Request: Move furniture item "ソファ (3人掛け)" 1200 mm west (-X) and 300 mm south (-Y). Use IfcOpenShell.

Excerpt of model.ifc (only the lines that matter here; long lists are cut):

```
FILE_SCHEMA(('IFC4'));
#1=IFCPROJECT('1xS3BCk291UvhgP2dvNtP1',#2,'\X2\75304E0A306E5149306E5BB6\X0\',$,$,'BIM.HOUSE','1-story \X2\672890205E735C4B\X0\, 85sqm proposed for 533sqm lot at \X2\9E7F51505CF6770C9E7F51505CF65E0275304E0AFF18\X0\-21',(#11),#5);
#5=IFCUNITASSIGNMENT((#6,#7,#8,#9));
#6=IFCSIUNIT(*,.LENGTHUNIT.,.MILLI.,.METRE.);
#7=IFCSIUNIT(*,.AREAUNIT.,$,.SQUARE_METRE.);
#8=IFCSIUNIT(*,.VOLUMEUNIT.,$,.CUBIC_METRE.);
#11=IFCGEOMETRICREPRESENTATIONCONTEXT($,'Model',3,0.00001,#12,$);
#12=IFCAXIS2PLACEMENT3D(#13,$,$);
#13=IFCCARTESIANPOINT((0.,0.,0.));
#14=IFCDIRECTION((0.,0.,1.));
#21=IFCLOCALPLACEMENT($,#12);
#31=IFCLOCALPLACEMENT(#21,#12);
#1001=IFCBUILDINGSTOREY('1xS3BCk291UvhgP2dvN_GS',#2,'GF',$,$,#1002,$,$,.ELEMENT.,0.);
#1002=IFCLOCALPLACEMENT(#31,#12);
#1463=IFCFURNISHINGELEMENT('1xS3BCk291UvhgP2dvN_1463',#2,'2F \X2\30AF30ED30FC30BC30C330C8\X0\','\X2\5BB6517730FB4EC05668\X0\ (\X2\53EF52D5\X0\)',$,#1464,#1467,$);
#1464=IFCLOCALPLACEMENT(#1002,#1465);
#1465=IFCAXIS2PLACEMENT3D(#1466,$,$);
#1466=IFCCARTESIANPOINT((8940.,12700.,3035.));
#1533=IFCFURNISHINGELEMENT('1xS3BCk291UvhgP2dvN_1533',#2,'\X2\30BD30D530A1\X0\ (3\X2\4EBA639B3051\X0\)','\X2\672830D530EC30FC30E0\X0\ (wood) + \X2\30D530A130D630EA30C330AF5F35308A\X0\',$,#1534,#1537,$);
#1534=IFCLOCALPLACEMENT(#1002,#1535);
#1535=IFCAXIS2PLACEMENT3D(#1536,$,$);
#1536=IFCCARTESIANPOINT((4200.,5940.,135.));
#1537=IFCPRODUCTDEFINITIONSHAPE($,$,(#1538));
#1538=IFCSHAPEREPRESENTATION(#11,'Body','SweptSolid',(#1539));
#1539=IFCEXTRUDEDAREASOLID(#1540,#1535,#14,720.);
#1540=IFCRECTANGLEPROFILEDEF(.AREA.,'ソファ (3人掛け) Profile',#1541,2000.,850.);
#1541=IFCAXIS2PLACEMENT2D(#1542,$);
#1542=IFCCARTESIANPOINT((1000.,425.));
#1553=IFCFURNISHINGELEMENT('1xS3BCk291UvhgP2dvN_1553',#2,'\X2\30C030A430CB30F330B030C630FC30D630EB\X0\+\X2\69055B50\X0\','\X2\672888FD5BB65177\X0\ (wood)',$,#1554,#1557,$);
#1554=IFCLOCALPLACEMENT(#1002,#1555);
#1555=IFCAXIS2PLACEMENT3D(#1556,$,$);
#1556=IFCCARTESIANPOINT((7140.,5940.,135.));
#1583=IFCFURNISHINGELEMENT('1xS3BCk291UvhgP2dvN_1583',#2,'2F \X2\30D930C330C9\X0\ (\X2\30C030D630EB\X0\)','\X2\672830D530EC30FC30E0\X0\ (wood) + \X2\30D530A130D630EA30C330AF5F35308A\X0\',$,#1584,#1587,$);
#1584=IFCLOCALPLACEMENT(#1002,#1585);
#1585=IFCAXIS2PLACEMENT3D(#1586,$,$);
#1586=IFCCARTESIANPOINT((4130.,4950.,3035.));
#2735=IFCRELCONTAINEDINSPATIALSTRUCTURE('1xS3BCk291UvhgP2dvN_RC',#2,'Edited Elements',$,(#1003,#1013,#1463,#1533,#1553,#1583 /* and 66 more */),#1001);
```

```python
import ifcopenshell
import ifcopenshell.api.geometry
import ifcopenshell.util.placement
import ifcopenshell.util.unit

model = ifcopenshell.open("model.ifc")
unit_scale = ifcopenshell.util.unit.calculate_unit_scale(model)

item = model.by_guid("1xS3BCk291UvhgP2dvN_1533")
matrix = ifcopenshell.util.placement.get_local_placement(item.ObjectPlacement)
matrix[0, 3] -= 1.2 / unit_scale
matrix[1, 3] -= 0.3 / unit_scale
ifcopenshell.api.geometry.edit_object_placement(model, product=item, matrix=matrix, is_si=False)

print(ifcopenshell.util.placement.get_local_placement(item.ObjectPlacement).round(3) + 0.0)

model.write("model_edited.ifc")
```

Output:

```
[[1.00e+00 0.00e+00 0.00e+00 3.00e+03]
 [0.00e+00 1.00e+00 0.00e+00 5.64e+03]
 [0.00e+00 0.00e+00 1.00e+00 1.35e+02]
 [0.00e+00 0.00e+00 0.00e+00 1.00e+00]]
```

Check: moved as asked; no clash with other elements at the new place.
